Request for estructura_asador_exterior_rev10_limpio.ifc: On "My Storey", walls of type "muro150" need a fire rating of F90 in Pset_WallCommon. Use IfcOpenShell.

First a look at what the model holds.

```python
import ifcopenshell
import ifcopenshell.util.element

model = ifcopenshell.open("estructura_asador_exterior_rev10_limpio.ifc")
print(model.schema)
storey = next(s for s in model.by_type("IfcBuildingStorey") if s.Name == "My Storey")
walls = [e for e in ifcopenshell.util.element.get_decomposition(storey) if e.is_a("IfcWall")]
seen = {}
for e in walls:
    element_type = ifcopenshell.util.element.get_type(e)
    key = (element_type.Name if element_type != e and element_type else None, ifcopenshell.util.element.get_pset(e, "Pset_WallCommon", "FireRating"))
    seen[key] = seen.get(key, 0) + 1
for (name, value), count in sorted(seen.items(), key=str):
    print(count, "x", name, "|", value)
```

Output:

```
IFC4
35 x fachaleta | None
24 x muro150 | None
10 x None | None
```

```python
import ifcopenshell
import ifcopenshell.api.pset
import ifcopenshell.util.element

model = ifcopenshell.open("estructura_asador_exterior_rev10_limpio.ifc")

storey = next(s for s in model.by_type("IfcBuildingStorey") if s.Name == "My Storey")
walls = [e for e in ifcopenshell.util.element.get_decomposition(storey) if e.is_a("IfcWall")]

count = 0
for e in walls:
    element_type = ifcopenshell.util.element.get_type(e)
    if element_type in (None, e) or element_type.Name != "muro150":
        continue
    # add_pset returns the element's existing set when there is one.
    pset = ifcopenshell.api.pset.add_pset(model, product=e, name="Pset_WallCommon")
    ifcopenshell.api.pset.edit_pset(model, pset=pset, properties={"FireRating": "F90"})
    count += 1

print(count, "walls updated")

model.write("estructura_asador_exterior_rev10_limpio_updated.ifc")
```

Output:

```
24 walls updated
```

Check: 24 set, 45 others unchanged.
